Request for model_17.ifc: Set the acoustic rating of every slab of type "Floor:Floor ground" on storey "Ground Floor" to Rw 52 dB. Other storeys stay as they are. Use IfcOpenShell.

First a look at what the model holds.

```python
import ifcopenshell
import ifcopenshell.util.element

model = ifcopenshell.open("model_17.ifc")
print(model.schema)
storey = next(s for s in model.by_type("IfcBuildingStorey") if s.Name == "Ground Floor")
slabs = [e for e in ifcopenshell.util.element.get_decomposition(storey) if e.is_a("IfcSlab")]
seen = {}
for e in slabs:
    element_type = ifcopenshell.util.element.get_type(e)
    key = (element_type.Name if element_type != e and element_type else None, ifcopenshell.util.element.get_pset(e, "Pset_SlabCommon", "AcousticRating"))
    seen[key] = seen.get(key, 0) + 1
for (name, value), count in sorted(seen.items(), key=str):
    print(count, "x", name, "|", value)
```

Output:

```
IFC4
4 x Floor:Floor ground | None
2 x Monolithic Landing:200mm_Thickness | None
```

```python
import ifcopenshell
import ifcopenshell.api.pset
import ifcopenshell.util.element

model = ifcopenshell.open("model_17.ifc")

storey = next(s for s in model.by_type("IfcBuildingStorey") if s.Name == "Ground Floor")
slabs = [e for e in ifcopenshell.util.element.get_decomposition(storey) if e.is_a("IfcSlab")]

count = 0
for e in slabs:
    element_type = ifcopenshell.util.element.get_type(e)
    if element_type in (None, e) or element_type.Name != "Floor:Floor ground":
        continue
    # add_pset returns the element's existing set when there is one.
    pset = ifcopenshell.api.pset.add_pset(model, product=e, name="Pset_SlabCommon")
    ifcopenshell.api.pset.edit_pset(model, pset=pset, properties={"AcousticRating": "Rw 52 dB"})
    count += 1

print(count, "slabs updated")

model.write("model_17_edited.ifc")
```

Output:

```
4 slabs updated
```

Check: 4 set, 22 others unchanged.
